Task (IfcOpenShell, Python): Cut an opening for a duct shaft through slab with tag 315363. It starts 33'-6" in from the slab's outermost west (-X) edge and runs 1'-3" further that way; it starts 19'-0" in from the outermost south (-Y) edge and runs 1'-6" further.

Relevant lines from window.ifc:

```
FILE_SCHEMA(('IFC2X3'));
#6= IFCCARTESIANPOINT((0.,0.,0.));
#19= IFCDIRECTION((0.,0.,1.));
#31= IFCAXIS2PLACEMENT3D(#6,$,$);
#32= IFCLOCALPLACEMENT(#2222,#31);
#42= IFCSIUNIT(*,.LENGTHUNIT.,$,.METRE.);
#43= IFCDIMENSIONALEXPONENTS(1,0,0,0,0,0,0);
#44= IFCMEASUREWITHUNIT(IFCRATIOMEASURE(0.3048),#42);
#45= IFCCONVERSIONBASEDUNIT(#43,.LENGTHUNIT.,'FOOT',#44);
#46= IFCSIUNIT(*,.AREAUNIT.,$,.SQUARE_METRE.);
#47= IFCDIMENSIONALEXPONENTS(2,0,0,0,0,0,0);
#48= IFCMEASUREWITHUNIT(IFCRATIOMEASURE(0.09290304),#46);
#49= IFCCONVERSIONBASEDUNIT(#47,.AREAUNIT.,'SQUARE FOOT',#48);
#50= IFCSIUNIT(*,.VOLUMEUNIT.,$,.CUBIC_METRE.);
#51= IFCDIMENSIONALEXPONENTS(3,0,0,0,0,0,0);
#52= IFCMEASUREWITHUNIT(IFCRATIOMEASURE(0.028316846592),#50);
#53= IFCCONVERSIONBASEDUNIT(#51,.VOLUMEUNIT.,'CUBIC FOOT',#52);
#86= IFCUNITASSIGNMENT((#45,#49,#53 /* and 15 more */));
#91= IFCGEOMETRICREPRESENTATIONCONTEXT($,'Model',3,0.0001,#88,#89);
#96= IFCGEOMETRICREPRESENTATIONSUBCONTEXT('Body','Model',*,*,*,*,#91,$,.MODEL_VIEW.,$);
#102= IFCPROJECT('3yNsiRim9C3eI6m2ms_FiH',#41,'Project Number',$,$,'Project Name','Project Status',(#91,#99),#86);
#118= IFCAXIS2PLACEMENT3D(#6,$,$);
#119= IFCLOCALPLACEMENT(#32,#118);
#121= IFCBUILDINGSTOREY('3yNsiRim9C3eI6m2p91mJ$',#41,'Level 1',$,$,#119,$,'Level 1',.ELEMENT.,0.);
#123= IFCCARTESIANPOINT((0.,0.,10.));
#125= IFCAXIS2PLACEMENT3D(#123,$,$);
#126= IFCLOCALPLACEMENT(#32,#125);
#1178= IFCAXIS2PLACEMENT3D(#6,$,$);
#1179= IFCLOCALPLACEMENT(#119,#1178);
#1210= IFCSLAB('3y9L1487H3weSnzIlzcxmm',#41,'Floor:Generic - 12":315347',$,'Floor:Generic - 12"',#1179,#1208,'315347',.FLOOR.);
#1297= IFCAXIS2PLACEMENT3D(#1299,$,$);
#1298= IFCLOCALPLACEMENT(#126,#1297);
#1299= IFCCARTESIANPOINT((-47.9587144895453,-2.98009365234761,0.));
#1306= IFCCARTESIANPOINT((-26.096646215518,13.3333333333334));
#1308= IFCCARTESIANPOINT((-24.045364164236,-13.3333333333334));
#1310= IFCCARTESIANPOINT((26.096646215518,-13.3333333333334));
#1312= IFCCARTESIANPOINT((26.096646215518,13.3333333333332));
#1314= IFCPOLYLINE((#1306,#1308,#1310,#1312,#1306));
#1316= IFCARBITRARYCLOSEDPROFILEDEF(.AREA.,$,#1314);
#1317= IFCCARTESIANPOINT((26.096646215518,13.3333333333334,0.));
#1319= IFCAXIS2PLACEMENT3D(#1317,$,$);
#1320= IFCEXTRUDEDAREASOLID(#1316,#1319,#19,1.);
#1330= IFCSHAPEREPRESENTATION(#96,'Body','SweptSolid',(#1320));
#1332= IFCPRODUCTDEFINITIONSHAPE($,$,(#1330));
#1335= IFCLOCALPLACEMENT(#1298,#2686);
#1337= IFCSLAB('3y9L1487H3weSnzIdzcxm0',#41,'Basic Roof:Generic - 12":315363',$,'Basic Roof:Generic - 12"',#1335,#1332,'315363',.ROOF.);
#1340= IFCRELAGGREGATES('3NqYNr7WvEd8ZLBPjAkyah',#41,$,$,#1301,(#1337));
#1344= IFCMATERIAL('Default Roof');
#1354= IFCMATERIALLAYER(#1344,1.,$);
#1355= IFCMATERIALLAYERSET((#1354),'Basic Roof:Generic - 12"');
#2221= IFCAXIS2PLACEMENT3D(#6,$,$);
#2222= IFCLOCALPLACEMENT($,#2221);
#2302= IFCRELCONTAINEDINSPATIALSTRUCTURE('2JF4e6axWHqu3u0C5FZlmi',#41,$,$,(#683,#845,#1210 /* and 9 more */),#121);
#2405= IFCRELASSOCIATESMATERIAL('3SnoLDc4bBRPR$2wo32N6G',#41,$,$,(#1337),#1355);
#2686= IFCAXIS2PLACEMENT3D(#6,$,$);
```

```python
import numpy as np
import ifcopenshell
import ifcopenshell.api.feature
import ifcopenshell.api.geometry
import ifcopenshell.api.root
import ifcopenshell.geom
import ifcopenshell.util.placement
import ifcopenshell.util.representation
import ifcopenshell.util.shape
import ifcopenshell.util.unit

model = ifcopenshell.open("window.ifc")
unit_scale = ifcopenshell.util.unit.calculate_unit_scale(model)
settings = ifcopenshell.geom.settings()


def volume(element):
    """Net volume in cubic metres, openings subtracted."""
    shape = ifcopenshell.geom.create_shape(settings, element)
    return ifcopenshell.util.shape.get_volume(shape.geometry)


slab = model.by_id(1337)
before = volume(slab)

# Extent in the slab's own axes, in metres. The edges named are its -X and -Y sides.
slab_shape = ifcopenshell.geom.create_shape(settings, slab)
vertices = ifcopenshell.util.shape.get_vertices(slab_shape.geometry)
x_min, y_min, bottom = vertices.min(axis=0)
top = vertices[:, 2].max()

opening = ifcopenshell.api.root.create_entity(model, ifc_class="IfcOpeningElement", name="Duct shaft opening")
context = ifcopenshell.util.representation.get_context(model, "Model", "Body", "MODEL_VIEW")
width, depth = 0.381, 0.4572
outline = [(0.0, 0.0), (width, 0.0), (width, depth), (0.0, depth), (0.0, 0.0)]
# Overshoot both faces by 50 mm so the cut is clean.
shape = ifcopenshell.api.geometry.add_slab_representation(
    model, context=context, depth=top - bottom + 0.1, polyline=outline
)
ifcopenshell.api.geometry.assign_representation(model, product=opening, representation=shape)

matrix = ifcopenshell.util.placement.get_local_placement(slab.ObjectPlacement)
matrix[:, 3] = matrix @ np.append(np.array([x_min + 10.2108, y_min + 5.7912, bottom - 0.05]) / unit_scale, 1.0)
ifcopenshell.api.geometry.edit_object_placement(model, product=opening, matrix=matrix, is_si=False)
ifcopenshell.api.feature.add_feature(model, feature=opening, element=slab)

after = volume(slab)

print(f"slab volume {before:.3f} -> {after:.3f} m3")

model.write("window_v2.ifc")
```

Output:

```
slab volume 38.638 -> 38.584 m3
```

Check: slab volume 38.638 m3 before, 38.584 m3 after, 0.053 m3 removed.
